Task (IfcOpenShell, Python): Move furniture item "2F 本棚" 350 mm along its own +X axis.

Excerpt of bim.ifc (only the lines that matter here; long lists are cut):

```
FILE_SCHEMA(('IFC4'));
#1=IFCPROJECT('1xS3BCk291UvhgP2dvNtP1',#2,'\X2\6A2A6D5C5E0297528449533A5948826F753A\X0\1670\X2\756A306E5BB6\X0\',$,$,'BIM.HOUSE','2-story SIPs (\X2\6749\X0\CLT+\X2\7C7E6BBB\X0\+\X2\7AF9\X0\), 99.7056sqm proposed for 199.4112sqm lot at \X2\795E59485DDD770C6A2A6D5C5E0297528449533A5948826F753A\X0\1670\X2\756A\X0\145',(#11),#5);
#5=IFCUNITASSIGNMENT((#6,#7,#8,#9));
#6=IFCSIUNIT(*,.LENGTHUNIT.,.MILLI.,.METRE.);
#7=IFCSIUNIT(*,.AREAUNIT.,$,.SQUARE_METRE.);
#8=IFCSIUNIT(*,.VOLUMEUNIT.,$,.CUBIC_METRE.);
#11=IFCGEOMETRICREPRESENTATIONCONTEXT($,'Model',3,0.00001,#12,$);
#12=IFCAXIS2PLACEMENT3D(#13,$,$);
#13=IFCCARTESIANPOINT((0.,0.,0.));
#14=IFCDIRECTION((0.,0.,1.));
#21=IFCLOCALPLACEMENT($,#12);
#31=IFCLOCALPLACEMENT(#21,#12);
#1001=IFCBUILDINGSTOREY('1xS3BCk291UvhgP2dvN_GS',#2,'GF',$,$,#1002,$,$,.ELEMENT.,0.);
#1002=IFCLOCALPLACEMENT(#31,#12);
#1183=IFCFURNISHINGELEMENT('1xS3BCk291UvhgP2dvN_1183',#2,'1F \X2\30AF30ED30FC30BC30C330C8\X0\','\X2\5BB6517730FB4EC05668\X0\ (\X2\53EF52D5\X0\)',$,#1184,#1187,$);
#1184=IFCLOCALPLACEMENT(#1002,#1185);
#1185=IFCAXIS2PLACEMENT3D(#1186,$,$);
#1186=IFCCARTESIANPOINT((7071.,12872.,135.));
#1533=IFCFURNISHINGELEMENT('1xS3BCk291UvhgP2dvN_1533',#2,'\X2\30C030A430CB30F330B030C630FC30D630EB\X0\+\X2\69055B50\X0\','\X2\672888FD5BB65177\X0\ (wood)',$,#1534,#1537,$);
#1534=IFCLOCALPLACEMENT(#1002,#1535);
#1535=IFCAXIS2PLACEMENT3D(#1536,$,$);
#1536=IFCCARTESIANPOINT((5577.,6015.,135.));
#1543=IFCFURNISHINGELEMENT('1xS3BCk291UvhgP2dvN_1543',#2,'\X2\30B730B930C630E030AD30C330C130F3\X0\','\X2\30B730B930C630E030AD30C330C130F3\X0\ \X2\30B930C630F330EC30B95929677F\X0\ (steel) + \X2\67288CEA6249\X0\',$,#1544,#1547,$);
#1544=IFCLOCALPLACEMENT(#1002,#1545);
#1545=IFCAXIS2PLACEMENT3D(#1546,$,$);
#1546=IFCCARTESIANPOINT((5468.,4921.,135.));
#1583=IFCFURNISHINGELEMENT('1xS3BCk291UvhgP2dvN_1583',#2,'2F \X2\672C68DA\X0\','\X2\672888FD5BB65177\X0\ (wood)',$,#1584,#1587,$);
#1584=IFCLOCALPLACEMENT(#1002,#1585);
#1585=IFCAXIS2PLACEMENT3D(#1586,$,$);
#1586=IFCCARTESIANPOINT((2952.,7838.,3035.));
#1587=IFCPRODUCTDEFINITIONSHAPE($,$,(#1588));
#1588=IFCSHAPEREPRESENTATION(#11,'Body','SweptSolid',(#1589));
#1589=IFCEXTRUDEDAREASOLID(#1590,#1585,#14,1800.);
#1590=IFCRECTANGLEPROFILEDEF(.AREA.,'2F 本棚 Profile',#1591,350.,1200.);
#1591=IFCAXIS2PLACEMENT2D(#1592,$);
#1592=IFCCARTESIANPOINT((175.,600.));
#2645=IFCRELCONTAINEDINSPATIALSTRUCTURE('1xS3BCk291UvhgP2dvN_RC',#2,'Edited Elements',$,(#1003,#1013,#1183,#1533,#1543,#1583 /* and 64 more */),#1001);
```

```python
import ifcopenshell
import ifcopenshell.api.geometry
import ifcopenshell.util.placement

model = ifcopenshell.open("bim.ifc")

item = model.by_id(1583)
matrix = ifcopenshell.util.placement.get_local_placement(item.ObjectPlacement)
matrix[:3, 3] += matrix[:3, 0] * 350.0
ifcopenshell.api.geometry.edit_object_placement(model, product=item, matrix=matrix, is_si=False)

print(ifcopenshell.util.placement.get_local_placement(item.ObjectPlacement).round(3) + 0.0)

model.write("bim_rev.ifc")
```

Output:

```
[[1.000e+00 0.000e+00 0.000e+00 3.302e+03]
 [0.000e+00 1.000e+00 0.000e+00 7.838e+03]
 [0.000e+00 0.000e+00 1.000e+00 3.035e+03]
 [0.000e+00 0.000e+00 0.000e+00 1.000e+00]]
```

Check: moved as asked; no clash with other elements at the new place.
